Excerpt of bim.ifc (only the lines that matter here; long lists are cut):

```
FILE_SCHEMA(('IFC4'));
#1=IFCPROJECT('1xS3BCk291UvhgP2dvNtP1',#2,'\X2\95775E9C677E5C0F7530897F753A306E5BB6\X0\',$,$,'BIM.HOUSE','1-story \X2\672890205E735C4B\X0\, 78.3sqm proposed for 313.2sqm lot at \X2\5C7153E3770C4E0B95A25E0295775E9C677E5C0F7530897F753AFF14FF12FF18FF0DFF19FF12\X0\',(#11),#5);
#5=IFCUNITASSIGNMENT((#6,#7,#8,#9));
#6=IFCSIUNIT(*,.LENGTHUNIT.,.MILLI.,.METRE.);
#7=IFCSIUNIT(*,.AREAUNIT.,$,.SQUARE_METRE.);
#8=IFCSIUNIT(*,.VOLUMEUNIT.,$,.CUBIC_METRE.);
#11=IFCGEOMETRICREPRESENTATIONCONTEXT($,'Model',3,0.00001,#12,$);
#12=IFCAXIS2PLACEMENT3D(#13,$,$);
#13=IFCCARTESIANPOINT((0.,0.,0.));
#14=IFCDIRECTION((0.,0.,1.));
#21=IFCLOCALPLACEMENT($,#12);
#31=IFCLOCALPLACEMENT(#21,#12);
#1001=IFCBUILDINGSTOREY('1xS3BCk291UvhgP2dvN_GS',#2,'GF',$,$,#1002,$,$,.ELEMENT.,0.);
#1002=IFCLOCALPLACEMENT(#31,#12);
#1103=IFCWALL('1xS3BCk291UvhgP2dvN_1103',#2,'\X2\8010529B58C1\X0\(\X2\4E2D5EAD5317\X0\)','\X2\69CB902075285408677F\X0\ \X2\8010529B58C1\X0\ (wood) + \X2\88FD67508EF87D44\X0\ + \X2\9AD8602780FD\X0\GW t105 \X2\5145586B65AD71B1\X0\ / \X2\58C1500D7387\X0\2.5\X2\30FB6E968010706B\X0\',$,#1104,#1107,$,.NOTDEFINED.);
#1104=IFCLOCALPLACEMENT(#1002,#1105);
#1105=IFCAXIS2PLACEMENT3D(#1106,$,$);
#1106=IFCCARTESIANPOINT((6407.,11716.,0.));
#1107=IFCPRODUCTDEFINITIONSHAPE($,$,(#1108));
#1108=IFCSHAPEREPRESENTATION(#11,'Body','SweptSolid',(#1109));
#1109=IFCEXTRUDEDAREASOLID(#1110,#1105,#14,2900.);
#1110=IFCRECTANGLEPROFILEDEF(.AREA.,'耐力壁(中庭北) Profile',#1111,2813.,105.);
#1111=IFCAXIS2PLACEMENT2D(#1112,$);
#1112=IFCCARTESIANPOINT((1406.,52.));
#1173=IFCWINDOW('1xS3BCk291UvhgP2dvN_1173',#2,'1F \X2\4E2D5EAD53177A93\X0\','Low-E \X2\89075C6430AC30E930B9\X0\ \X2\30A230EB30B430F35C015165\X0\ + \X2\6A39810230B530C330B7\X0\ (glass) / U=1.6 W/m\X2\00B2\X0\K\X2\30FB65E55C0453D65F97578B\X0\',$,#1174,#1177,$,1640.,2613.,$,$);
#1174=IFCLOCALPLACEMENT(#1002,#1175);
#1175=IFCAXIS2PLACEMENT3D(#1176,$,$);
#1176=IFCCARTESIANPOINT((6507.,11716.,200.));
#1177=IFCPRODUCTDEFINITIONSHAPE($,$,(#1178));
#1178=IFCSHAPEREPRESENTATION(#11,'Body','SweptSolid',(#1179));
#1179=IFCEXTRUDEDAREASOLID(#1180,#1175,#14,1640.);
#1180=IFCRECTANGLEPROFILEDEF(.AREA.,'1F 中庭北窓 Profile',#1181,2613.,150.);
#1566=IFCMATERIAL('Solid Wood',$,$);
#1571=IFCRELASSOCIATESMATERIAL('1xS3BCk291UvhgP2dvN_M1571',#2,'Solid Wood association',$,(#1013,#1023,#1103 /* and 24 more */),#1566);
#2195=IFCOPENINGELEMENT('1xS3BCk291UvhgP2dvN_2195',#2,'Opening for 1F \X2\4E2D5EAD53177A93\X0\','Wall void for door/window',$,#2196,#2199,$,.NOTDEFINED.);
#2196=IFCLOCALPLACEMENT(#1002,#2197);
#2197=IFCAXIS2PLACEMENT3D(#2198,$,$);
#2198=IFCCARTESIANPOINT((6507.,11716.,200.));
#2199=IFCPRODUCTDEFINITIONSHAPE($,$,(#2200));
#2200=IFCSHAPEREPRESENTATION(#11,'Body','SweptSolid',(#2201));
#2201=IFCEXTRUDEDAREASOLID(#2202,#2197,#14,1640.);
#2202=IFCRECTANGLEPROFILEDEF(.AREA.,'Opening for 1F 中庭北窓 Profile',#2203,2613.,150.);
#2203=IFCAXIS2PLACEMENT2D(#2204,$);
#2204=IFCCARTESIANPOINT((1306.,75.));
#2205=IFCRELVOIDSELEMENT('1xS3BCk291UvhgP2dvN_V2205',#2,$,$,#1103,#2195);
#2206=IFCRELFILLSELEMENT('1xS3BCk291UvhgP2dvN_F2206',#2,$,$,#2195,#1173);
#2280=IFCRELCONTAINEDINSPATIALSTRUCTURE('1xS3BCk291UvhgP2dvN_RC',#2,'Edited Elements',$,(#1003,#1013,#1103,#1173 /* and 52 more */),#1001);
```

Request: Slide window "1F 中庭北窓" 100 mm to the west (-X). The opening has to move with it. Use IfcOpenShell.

```python
import ifcopenshell
import ifcopenshell.api.geometry
import ifcopenshell.util.placement

model = ifcopenshell.open("bim.ifc")

window = model.by_guid("1xS3BCk291UvhgP2dvN_1173")
opening = window.FillsVoids[0].RelatingOpeningElement
wall = opening.VoidsElements[0].RelatingBuildingElement

wall_matrix = ifcopenshell.util.placement.get_local_placement(wall.ObjectPlacement)
shift = wall_matrix[:3, 0] * -100.0
before = ifcopenshell.util.placement.get_local_placement(window.ObjectPlacement)[:3, 3].copy()

# The window is not placed relative to its opening, so move both.
for product in (opening, window):
    matrix = ifcopenshell.util.placement.get_local_placement(product.ObjectPlacement)
    matrix[:3, 3] += shift
    ifcopenshell.api.geometry.edit_object_placement(model, product=product, matrix=matrix, is_si=False)

after = ifcopenshell.util.placement.get_local_placement(window.ObjectPlacement)[:3, 3]
print("window moved by", (after - before).round(3) + 0.0)

model.write("bim_edited.ifc")
```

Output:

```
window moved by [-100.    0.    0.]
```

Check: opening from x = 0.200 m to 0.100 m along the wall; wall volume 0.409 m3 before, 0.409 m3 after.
